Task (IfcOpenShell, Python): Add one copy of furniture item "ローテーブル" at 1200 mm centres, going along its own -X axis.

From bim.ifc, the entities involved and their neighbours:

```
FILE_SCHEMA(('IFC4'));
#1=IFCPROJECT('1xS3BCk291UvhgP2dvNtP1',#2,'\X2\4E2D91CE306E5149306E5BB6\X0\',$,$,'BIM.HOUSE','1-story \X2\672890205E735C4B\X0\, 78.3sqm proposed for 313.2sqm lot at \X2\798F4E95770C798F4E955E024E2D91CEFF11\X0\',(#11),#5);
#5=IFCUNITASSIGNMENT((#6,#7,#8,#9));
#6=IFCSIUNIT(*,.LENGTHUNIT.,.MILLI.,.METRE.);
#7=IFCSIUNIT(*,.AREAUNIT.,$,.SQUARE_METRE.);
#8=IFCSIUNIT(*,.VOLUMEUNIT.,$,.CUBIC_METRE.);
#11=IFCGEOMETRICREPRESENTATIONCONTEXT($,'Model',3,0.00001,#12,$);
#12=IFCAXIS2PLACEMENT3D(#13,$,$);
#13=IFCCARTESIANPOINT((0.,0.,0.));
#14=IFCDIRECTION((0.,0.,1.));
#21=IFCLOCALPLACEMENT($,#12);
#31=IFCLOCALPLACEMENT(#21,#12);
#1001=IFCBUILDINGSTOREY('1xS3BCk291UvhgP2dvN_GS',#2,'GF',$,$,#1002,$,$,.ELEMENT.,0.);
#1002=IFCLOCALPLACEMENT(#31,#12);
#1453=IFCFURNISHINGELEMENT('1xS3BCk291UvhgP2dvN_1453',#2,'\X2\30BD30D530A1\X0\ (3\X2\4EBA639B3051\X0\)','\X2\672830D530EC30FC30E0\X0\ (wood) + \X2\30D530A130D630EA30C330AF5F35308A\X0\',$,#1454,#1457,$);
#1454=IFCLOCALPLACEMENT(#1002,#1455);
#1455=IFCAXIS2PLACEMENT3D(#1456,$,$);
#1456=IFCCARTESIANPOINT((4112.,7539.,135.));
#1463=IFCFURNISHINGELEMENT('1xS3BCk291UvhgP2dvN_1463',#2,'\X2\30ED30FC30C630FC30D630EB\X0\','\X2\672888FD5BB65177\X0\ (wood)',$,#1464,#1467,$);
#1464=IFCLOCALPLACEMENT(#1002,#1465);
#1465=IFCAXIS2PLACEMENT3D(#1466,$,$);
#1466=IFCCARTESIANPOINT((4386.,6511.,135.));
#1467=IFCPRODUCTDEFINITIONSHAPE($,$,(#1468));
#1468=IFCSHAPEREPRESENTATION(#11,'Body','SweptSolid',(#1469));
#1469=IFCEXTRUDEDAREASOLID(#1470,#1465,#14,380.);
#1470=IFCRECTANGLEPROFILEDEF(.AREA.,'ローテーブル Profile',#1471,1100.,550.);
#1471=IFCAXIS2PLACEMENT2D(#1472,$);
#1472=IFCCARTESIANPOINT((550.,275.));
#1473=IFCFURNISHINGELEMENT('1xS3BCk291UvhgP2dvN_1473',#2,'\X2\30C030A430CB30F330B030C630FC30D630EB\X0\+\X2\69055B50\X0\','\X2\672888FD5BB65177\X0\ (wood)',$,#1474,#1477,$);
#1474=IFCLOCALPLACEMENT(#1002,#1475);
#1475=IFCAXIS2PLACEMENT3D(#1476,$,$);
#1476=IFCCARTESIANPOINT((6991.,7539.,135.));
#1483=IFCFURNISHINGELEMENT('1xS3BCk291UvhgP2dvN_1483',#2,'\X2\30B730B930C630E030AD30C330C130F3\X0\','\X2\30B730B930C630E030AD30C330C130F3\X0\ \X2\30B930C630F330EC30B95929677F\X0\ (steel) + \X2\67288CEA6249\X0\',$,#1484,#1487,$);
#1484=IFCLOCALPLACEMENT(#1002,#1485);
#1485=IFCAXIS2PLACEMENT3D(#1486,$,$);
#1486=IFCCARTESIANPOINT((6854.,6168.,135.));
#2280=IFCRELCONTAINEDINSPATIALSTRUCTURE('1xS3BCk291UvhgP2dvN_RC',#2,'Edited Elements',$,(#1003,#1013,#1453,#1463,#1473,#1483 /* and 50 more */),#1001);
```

```python
import ifcopenshell
import ifcopenshell.api.geometry
import ifcopenshell.api.root
import ifcopenshell.util.element
import ifcopenshell.util.placement
import ifcopenshell.util.unit

model = ifcopenshell.open("bim.ifc")
unit_scale = ifcopenshell.util.unit.calculate_unit_scale(model)


def reuse_history(source, copy):
    """copy_class also copies each property set's owner history, people and application; keep the originals."""
    for rel in copy.IsDefinedBy:
        if rel.is_a("IfcRelDefinesByProperties") and (history := rel.RelatingPropertyDefinition.OwnerHistory):
            rel.RelatingPropertyDefinition.OwnerHistory = source.OwnerHistory
            ifcopenshell.util.element.remove_deep2(model, history)


source = model.by_id(1463)
base = ifcopenshell.util.placement.get_local_placement(source.ObjectPlacement)
step = -base[:3, 0] * 1.2 / unit_scale

for i in range(1, 2):
    copy = ifcopenshell.api.root.copy_class(model, product=source)
    copy.Representation = ifcopenshell.util.element.copy_deep(
        model, source.Representation, exclude=["IfcGeometricRepresentationContext", "IfcRepresentationMap"]
    )
    reuse_history(source, copy)
    matrix = base.copy()
    matrix[:3, 3] += i * step
    print("added at", matrix[:3, 3].round(3) + 0.0)
    ifcopenshell.api.geometry.edit_object_placement(model, product=copy, matrix=matrix, is_si=False)

model.write("bim_v2.ifc")
```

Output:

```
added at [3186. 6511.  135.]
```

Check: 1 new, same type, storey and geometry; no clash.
